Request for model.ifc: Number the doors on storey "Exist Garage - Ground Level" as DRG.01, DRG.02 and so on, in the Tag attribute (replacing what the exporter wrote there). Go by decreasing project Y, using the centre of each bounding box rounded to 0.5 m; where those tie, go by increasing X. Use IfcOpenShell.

First a look at what the model holds.

```python
import ifcopenshell
import ifcopenshell.util.element
import ifcopenshell.util.placement

model = ifcopenshell.open("model.ifc")
print(model.schema)
storey = next(s for s in model.by_type("IfcBuildingStorey") if s.Name == "Exist Garage - Ground Level")
doors = [e for e in ifcopenshell.util.element.get_decomposition(storey) if e.is_a("IfcDoor")]
for e in sorted(doors, key=lambda e: e.id()):
    origin = ifcopenshell.util.placement.get_local_placement(e.ObjectPlacement)[:3, 3]
    print(e.id(), e.Tag, e.Name, origin.round(2) + 0.0, sep=" | ")
```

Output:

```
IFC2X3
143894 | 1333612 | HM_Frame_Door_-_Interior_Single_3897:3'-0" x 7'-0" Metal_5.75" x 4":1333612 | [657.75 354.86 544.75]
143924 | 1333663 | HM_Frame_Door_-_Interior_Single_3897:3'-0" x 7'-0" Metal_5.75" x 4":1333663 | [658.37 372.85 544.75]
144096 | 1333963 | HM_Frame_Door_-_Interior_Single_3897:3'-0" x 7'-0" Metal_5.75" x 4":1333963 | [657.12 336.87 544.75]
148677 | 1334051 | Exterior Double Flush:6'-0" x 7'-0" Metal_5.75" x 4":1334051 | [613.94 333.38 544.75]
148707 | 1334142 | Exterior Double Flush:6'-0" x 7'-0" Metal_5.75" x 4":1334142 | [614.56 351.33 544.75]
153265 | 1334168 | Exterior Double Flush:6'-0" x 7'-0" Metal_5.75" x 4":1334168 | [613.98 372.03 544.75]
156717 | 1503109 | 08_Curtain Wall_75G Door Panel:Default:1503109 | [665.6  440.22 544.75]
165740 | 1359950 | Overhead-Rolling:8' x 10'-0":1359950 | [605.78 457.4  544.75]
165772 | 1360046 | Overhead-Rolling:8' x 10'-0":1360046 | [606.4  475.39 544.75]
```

```python
import ifcopenshell
import ifcopenshell.geom
import ifcopenshell.util.element
import ifcopenshell.util.shape

model = ifcopenshell.open("model.ifc")
settings = ifcopenshell.geom.settings()
settings.set("use-world-coords", True)


def centre(element):
    shape = ifcopenshell.geom.create_shape(settings, element)
    return ifcopenshell.util.shape.get_bbox_centroid(shape.geometry)


storey = next(s for s in model.by_type("IfcBuildingStorey") if s.Name == "Exist Garage - Ground Level")
doors = [e for e in ifcopenshell.util.element.get_decomposition(storey) if e.is_a("IfcDoor")]

# Insertion points can sit at a corner or the storey origin, so sort by the geometry (in metres).
centres = {e: centre(e) for e in doors}
doors.sort(key=lambda e: (-round(centres[e][1] / 0.5), centres[e][0]))

for i, e in enumerate(doors, start=1):
    number = f"DRG.{i:02d}"
    e.Tag = number
    print(e.id(), number)

model.write("model_updated.ifc")
```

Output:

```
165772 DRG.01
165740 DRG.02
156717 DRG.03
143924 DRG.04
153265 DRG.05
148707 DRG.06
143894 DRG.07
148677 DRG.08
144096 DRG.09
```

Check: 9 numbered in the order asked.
